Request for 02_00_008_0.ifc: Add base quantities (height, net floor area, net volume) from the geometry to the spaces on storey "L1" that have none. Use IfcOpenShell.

First a look at what the model holds.

```python
import ifcopenshell
import ifcopenshell.util.element
import ifcopenshell.util.unit

model = ifcopenshell.open("02_00_008_0.ifc")
print(model.schema)
for unit_type in ("LENGTHUNIT", "AREAUNIT", "VOLUMEUNIT"):
    print(unit_type, ifcopenshell.util.unit.calculate_unit_scale(model, unit_type))
storey = next(s for s in model.by_type("IfcBuildingStorey") if s.Name == "L1")
spaces = [e for e in ifcopenshell.util.element.get_decomposition(storey) if e.is_a("IfcSpace")]
for e in sorted(spaces, key=lambda e: e.id()):
    print(e.id(), e.is_a(), e.Name, list(ifcopenshell.util.element.get_psets(e, qtos_only=True)), sep=" | ")
```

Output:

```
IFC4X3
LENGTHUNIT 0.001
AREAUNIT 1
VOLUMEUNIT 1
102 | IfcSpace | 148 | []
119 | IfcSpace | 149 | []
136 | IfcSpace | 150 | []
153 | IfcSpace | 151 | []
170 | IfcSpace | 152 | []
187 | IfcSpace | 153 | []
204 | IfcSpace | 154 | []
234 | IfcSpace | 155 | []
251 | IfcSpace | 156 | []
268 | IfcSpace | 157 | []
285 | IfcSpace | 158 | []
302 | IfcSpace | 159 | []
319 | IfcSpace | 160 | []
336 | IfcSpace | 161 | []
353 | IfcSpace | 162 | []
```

```python
import ifcopenshell
import ifcopenshell.api.pset
import ifcopenshell.geom
import ifcopenshell.util.element
import ifcopenshell.util.shape
import ifcopenshell.util.unit

model = ifcopenshell.open("02_00_008_0.ifc")
unit_scale = ifcopenshell.util.unit.calculate_unit_scale(model)
area_scale = ifcopenshell.util.unit.calculate_unit_scale(model, "AREAUNIT")
volume_scale = ifcopenshell.util.unit.calculate_unit_scale(model, "VOLUMEUNIT")
settings = ifcopenshell.geom.settings()

storey = next(s for s in model.by_type("IfcBuildingStorey") if s.Name == "L1")
spaces = [e for e in ifcopenshell.util.element.get_decomposition(storey) if e.is_a("IfcSpace")]

for e in sorted(spaces, key=lambda e: e.id()):
    if ifcopenshell.util.element.get_psets(e, qtos_only=True, should_inherit=False):
        continue
    # Geometry comes back in metres, in the element's own axes.
    shape = ifcopenshell.geom.create_shape(settings, e)
    values = {
        "Height": ifcopenshell.util.shape.get_z(shape.geometry) / unit_scale,
        "NetFloorArea": ifcopenshell.util.shape.get_footprint_area(shape.geometry) / area_scale,
        "NetVolume": ifcopenshell.util.shape.get_volume(shape.geometry) / volume_scale,
    }
    qto = ifcopenshell.api.pset.add_qto(model, product=e, name="Qto_SpaceBaseQuantities")
    ifcopenshell.api.pset.edit_qto(model, qto=qto, properties=values)
    print(e.id(), {k: round(v, 3) for k, v in values.items()})

model.write("02_00_008_0_v2.ifc")
```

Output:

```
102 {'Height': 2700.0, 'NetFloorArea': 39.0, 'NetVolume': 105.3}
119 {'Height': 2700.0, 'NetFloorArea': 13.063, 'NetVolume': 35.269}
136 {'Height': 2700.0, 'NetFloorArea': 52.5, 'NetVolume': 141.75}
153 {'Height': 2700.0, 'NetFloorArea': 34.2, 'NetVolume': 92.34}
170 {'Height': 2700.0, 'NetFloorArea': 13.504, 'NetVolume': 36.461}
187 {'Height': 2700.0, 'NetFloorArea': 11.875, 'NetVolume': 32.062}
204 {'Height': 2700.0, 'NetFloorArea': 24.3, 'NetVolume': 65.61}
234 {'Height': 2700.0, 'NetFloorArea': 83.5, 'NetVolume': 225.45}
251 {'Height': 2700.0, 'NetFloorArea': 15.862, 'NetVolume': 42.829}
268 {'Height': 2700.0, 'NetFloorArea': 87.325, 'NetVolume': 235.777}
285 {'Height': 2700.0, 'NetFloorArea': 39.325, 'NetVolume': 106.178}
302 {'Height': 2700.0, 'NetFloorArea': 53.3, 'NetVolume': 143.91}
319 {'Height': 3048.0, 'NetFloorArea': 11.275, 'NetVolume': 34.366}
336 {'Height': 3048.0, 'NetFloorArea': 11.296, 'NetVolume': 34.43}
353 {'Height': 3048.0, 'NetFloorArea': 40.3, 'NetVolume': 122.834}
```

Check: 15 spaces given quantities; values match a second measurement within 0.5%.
